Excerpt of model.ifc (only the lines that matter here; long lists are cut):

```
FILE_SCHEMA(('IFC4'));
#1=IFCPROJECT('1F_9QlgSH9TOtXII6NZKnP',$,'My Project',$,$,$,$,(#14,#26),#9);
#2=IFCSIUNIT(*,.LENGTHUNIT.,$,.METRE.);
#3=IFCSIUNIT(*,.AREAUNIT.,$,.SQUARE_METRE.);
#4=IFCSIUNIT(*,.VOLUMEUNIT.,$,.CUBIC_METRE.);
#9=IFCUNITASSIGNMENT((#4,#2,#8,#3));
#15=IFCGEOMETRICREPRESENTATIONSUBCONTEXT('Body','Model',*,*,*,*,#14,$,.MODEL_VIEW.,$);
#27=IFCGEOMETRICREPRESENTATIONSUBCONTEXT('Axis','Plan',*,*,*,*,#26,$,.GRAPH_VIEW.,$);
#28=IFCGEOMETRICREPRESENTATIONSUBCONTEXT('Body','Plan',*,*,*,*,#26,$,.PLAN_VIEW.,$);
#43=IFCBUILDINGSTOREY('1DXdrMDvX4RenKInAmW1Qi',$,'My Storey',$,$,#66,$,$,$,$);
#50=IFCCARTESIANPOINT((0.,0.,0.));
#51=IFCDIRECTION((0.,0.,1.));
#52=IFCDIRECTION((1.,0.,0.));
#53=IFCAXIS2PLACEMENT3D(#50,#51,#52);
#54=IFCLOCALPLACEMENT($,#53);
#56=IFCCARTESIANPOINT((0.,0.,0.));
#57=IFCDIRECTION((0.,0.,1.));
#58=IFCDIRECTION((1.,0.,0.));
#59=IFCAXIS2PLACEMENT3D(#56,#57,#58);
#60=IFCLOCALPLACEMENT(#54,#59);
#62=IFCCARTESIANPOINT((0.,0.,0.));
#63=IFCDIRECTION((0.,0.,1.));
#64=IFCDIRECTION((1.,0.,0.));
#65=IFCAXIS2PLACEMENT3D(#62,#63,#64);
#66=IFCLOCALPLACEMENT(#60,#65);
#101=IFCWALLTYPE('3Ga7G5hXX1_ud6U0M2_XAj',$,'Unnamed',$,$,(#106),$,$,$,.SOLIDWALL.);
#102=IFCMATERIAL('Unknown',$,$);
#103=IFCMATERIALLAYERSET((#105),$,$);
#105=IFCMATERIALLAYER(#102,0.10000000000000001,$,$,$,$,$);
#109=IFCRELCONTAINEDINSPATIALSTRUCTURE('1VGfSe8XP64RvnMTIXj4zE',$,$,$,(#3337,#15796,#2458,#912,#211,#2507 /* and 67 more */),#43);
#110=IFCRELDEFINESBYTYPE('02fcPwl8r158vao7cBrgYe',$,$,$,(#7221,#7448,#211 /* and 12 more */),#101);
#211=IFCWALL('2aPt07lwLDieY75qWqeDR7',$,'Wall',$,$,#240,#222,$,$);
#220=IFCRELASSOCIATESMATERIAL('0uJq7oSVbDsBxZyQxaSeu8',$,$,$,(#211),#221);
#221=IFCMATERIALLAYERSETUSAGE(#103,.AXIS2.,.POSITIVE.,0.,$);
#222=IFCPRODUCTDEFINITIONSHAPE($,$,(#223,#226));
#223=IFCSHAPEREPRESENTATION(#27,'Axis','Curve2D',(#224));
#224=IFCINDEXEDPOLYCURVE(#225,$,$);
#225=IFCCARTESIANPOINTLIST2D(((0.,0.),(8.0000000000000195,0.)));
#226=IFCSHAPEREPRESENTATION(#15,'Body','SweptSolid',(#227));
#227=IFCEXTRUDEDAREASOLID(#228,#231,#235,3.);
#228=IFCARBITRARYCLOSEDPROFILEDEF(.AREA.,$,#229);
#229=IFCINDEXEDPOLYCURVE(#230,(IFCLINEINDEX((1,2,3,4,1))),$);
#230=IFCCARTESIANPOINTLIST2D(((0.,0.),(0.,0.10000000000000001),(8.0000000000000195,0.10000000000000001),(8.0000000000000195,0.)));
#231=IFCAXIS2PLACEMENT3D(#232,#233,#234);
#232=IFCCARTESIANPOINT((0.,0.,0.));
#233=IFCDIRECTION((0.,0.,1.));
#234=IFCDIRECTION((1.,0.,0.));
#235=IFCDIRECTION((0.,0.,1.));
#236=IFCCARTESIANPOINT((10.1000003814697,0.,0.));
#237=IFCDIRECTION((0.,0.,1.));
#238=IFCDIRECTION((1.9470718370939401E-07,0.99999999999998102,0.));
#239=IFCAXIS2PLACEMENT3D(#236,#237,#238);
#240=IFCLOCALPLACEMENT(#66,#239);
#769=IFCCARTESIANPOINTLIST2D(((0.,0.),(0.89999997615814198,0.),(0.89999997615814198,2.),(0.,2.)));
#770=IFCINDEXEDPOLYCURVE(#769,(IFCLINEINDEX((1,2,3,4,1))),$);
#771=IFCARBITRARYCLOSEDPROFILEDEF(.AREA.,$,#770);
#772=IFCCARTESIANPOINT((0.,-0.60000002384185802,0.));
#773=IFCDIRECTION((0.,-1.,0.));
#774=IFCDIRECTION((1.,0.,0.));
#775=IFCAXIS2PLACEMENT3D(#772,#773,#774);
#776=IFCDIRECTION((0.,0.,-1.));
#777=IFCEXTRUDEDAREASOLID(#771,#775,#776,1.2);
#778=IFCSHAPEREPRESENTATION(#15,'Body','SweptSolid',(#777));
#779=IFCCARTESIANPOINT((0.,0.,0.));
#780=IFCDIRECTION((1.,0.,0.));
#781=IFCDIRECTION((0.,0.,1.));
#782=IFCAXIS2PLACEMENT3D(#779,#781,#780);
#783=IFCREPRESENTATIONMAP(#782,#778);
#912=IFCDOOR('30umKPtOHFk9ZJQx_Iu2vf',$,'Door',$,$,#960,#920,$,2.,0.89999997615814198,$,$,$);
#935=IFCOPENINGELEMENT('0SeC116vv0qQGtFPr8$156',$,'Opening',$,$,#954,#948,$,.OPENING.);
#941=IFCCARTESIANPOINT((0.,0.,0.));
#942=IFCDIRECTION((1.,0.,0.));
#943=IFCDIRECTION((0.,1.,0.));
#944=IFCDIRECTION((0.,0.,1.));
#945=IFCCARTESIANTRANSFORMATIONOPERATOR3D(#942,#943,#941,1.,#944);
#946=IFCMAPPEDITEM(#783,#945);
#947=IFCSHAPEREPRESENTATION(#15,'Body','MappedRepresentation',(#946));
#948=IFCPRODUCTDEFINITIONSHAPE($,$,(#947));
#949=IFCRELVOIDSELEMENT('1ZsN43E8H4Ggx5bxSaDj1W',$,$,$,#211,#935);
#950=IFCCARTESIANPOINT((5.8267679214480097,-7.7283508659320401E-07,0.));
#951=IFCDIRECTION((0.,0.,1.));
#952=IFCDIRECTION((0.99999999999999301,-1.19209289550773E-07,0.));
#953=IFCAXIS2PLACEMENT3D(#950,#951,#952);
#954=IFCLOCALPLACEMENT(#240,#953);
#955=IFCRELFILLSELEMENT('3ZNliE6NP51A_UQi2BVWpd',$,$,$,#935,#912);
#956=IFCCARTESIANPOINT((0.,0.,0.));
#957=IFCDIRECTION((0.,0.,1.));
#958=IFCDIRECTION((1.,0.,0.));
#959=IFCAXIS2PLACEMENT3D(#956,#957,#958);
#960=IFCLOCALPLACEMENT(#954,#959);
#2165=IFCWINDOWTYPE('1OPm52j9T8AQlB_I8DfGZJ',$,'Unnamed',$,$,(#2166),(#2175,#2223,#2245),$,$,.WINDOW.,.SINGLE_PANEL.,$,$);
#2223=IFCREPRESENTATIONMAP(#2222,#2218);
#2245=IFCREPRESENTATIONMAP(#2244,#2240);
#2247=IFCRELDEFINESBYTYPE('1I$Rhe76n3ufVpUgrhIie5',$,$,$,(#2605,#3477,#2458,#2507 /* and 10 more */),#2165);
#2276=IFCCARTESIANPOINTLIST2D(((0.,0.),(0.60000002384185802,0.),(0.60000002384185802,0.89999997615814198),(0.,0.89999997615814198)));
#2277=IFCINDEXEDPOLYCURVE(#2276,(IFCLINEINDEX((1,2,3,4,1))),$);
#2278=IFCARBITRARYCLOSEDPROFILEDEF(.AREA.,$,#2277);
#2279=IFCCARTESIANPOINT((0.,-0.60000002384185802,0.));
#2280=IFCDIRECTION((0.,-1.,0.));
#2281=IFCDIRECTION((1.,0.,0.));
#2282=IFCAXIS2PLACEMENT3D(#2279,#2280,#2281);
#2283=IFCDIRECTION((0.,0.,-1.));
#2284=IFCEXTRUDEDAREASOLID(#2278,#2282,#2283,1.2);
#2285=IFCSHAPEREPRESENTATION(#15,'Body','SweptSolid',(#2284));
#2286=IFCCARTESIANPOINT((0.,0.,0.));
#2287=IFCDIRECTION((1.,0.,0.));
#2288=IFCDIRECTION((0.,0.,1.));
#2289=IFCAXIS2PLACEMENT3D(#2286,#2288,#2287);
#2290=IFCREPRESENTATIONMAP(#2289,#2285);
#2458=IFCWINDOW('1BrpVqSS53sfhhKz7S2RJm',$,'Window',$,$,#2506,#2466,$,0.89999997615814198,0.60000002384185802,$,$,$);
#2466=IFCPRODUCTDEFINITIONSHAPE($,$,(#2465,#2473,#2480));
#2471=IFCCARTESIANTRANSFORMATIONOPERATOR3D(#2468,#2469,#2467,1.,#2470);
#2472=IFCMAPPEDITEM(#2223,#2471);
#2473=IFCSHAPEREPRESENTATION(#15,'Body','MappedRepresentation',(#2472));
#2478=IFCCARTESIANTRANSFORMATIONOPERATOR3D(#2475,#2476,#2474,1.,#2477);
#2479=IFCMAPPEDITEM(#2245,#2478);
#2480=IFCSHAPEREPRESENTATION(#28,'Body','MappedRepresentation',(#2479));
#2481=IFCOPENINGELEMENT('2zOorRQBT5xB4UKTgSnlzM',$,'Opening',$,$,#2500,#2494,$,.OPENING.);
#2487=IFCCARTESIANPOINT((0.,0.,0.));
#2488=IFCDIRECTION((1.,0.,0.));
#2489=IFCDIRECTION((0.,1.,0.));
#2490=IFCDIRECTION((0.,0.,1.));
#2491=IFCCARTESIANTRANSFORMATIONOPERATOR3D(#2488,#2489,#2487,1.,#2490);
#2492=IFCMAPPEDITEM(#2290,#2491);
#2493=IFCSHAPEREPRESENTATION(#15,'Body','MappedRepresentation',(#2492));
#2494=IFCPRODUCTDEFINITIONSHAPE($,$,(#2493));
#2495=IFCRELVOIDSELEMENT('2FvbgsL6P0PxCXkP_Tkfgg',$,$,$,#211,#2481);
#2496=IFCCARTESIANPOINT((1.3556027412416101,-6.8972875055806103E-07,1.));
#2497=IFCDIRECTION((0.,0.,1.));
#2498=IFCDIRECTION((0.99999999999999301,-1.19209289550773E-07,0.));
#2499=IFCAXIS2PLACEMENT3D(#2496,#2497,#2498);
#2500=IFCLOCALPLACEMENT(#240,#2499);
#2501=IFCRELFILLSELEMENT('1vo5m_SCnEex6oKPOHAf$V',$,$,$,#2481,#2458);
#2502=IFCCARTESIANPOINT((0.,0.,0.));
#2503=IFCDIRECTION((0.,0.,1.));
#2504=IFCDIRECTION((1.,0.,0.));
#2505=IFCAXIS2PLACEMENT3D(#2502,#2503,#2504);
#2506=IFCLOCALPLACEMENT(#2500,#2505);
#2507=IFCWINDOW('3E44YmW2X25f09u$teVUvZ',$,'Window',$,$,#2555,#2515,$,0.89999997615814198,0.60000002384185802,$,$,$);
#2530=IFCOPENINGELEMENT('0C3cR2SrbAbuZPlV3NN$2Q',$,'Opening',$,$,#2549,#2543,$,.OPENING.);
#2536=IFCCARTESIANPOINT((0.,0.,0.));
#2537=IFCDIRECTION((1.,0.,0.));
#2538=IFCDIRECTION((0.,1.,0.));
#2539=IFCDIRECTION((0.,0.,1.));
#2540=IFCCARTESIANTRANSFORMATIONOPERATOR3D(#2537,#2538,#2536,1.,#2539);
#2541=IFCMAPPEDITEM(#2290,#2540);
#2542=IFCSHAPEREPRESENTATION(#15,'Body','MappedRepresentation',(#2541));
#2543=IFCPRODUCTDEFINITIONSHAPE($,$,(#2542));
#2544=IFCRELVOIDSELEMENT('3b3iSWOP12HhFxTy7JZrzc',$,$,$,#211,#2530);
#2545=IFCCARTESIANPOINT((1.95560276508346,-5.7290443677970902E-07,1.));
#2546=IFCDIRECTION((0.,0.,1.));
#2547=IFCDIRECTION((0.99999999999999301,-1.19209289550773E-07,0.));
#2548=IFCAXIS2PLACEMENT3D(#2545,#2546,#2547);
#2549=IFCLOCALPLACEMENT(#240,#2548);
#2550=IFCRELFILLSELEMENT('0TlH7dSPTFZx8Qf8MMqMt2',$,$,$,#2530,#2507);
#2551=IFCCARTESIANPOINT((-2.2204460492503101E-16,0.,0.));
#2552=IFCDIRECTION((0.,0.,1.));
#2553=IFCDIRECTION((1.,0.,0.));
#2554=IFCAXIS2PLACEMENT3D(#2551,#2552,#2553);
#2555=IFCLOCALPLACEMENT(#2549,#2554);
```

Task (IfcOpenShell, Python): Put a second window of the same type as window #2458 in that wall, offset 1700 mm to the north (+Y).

```python
import ifcopenshell
import ifcopenshell.api.feature
import ifcopenshell.api.geometry
import ifcopenshell.api.root
import ifcopenshell.geom
import ifcopenshell.util.element
import ifcopenshell.util.placement
import ifcopenshell.util.shape

model = ifcopenshell.open("model.ifc")
settings = ifcopenshell.geom.settings()


def volume(element):
    """Net volume in cubic metres, openings subtracted."""
    shape = ifcopenshell.geom.create_shape(settings, element)
    return ifcopenshell.util.shape.get_volume(shape.geometry)


window = model.by_id(2458)
opening = window.FillsVoids[0].RelatingOpeningElement
wall = opening.VoidsElements[0].RelatingBuildingElement
before = volume(wall)
shift = ifcopenshell.util.placement.get_local_placement(wall.ObjectPlacement)[:3, 0] * 1.7

# copy_class copies the void relationship, type, container and properties, but no geometry.
new_opening = ifcopenshell.api.root.copy_class(model, product=opening)
new_opening.Representation = ifcopenshell.util.element.copy_deep(
    model, opening.Representation, exclude=["IfcGeometricRepresentationContext", "IfcRepresentationMap"]
)
new_window = ifcopenshell.api.root.copy_class(model, product=window)
new_window.Representation = ifcopenshell.util.element.copy_deep(
    model, window.Representation, exclude=["IfcGeometricRepresentationContext", "IfcRepresentationMap"]
)
ifcopenshell.api.feature.add_filling(model, opening=new_opening, element=new_window)

for old, new in ((opening, new_opening), (window, new_window)):
    matrix = ifcopenshell.util.placement.get_local_placement(old.ObjectPlacement)
    matrix[:3, 3] += shift
    ifcopenshell.api.geometry.edit_object_placement(model, product=new, matrix=matrix, is_si=False)

after = volume(wall)

print(f"wall volume {before:.3f} -> {after:.3f} m3")

model.write("model-out.ifc")
```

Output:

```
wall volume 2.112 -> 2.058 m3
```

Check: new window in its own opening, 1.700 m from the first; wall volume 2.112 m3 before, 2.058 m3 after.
